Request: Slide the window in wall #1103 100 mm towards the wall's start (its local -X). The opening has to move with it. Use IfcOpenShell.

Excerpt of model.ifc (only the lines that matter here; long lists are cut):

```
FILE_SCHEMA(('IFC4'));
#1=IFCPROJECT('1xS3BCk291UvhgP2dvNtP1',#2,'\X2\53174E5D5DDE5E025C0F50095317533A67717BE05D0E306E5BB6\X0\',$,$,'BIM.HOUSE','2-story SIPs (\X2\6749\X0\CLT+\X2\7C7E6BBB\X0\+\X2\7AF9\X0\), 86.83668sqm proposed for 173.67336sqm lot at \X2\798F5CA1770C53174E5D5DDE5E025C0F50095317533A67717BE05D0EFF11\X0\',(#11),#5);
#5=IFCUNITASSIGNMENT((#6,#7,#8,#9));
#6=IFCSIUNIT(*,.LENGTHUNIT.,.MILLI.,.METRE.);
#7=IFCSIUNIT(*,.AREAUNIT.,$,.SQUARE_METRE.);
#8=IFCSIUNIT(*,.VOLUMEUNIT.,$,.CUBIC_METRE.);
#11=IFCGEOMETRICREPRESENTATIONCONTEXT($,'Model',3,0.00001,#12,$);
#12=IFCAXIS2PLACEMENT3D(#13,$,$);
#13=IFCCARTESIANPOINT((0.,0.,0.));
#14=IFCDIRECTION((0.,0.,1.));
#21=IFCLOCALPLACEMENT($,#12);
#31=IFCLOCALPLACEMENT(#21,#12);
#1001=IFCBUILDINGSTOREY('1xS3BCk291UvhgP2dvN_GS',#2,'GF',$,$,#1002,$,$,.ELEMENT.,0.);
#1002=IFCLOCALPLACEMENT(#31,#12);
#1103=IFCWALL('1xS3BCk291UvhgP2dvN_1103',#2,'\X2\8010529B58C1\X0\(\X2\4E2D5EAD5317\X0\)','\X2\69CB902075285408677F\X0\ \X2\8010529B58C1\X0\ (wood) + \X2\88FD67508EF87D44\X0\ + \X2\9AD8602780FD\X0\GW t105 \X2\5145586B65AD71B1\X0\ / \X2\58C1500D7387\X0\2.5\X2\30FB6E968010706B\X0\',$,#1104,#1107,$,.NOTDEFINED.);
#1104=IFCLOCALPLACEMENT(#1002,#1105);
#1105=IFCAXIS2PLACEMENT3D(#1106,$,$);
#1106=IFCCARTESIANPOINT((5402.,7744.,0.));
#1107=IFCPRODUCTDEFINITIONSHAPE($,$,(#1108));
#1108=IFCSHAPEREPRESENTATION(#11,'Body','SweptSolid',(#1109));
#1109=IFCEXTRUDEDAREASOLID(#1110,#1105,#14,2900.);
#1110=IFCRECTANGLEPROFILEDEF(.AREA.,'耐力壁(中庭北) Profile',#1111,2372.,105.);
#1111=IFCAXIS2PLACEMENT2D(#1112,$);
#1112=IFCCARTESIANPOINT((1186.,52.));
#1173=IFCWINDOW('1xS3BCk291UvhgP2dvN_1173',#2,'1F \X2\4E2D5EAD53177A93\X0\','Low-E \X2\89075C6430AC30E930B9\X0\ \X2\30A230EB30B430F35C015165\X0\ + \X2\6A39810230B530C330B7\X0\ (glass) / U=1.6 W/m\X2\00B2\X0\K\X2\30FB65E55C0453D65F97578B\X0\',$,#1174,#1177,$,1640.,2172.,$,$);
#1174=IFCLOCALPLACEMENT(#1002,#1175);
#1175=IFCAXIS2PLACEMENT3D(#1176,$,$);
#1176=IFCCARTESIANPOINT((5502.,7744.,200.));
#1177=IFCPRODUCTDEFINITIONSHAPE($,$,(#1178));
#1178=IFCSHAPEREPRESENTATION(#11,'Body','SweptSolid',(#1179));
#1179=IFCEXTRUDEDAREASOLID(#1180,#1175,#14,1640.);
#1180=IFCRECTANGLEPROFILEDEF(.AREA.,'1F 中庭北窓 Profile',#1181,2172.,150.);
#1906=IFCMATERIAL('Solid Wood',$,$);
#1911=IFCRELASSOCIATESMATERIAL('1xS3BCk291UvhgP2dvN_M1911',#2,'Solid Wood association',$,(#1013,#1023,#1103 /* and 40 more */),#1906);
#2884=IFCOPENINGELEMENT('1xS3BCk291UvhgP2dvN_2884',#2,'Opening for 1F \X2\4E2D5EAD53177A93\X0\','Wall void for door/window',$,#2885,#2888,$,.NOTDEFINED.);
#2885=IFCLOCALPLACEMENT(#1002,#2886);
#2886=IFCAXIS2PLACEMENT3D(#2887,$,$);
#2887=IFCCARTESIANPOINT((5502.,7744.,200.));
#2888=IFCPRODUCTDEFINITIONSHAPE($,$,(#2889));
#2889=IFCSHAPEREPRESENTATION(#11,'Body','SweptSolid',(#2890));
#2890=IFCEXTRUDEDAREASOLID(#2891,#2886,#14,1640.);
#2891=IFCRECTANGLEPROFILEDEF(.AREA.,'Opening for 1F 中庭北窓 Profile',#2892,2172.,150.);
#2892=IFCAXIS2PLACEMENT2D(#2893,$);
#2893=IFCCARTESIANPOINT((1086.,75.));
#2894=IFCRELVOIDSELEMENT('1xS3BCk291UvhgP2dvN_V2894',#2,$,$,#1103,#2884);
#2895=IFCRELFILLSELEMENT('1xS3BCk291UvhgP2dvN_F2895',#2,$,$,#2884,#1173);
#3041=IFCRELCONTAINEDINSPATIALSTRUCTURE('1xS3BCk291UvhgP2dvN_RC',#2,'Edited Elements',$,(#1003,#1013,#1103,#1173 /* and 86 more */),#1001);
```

```python
import ifcopenshell
import ifcopenshell.api.geometry
import ifcopenshell.util.placement
import ifcopenshell.util.unit

model = ifcopenshell.open("model.ifc")
unit_scale = ifcopenshell.util.unit.calculate_unit_scale(model)

window = model.by_guid("1xS3BCk291UvhgP2dvN_1173")
opening = window.FillsVoids[0].RelatingOpeningElement
wall = opening.VoidsElements[0].RelatingBuildingElement

wall_matrix = ifcopenshell.util.placement.get_local_placement(wall.ObjectPlacement)
shift = wall_matrix[:3, 0] * -0.1 / unit_scale
before = ifcopenshell.util.placement.get_local_placement(window.ObjectPlacement)[:3, 3].copy()

# The window is not placed relative to its opening, so move both.
for product in (opening, window):
    matrix = ifcopenshell.util.placement.get_local_placement(product.ObjectPlacement)
    matrix[:3, 3] += shift
    ifcopenshell.api.geometry.edit_object_placement(model, product=product, matrix=matrix, is_si=False)

after = ifcopenshell.util.placement.get_local_placement(window.ObjectPlacement)[:3, 3]
print("window moved by", (after - before).round(3) + 0.0)

model.write("model_v2.ifc")
```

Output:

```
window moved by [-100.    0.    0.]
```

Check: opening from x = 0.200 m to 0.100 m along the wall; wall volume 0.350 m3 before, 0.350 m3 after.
